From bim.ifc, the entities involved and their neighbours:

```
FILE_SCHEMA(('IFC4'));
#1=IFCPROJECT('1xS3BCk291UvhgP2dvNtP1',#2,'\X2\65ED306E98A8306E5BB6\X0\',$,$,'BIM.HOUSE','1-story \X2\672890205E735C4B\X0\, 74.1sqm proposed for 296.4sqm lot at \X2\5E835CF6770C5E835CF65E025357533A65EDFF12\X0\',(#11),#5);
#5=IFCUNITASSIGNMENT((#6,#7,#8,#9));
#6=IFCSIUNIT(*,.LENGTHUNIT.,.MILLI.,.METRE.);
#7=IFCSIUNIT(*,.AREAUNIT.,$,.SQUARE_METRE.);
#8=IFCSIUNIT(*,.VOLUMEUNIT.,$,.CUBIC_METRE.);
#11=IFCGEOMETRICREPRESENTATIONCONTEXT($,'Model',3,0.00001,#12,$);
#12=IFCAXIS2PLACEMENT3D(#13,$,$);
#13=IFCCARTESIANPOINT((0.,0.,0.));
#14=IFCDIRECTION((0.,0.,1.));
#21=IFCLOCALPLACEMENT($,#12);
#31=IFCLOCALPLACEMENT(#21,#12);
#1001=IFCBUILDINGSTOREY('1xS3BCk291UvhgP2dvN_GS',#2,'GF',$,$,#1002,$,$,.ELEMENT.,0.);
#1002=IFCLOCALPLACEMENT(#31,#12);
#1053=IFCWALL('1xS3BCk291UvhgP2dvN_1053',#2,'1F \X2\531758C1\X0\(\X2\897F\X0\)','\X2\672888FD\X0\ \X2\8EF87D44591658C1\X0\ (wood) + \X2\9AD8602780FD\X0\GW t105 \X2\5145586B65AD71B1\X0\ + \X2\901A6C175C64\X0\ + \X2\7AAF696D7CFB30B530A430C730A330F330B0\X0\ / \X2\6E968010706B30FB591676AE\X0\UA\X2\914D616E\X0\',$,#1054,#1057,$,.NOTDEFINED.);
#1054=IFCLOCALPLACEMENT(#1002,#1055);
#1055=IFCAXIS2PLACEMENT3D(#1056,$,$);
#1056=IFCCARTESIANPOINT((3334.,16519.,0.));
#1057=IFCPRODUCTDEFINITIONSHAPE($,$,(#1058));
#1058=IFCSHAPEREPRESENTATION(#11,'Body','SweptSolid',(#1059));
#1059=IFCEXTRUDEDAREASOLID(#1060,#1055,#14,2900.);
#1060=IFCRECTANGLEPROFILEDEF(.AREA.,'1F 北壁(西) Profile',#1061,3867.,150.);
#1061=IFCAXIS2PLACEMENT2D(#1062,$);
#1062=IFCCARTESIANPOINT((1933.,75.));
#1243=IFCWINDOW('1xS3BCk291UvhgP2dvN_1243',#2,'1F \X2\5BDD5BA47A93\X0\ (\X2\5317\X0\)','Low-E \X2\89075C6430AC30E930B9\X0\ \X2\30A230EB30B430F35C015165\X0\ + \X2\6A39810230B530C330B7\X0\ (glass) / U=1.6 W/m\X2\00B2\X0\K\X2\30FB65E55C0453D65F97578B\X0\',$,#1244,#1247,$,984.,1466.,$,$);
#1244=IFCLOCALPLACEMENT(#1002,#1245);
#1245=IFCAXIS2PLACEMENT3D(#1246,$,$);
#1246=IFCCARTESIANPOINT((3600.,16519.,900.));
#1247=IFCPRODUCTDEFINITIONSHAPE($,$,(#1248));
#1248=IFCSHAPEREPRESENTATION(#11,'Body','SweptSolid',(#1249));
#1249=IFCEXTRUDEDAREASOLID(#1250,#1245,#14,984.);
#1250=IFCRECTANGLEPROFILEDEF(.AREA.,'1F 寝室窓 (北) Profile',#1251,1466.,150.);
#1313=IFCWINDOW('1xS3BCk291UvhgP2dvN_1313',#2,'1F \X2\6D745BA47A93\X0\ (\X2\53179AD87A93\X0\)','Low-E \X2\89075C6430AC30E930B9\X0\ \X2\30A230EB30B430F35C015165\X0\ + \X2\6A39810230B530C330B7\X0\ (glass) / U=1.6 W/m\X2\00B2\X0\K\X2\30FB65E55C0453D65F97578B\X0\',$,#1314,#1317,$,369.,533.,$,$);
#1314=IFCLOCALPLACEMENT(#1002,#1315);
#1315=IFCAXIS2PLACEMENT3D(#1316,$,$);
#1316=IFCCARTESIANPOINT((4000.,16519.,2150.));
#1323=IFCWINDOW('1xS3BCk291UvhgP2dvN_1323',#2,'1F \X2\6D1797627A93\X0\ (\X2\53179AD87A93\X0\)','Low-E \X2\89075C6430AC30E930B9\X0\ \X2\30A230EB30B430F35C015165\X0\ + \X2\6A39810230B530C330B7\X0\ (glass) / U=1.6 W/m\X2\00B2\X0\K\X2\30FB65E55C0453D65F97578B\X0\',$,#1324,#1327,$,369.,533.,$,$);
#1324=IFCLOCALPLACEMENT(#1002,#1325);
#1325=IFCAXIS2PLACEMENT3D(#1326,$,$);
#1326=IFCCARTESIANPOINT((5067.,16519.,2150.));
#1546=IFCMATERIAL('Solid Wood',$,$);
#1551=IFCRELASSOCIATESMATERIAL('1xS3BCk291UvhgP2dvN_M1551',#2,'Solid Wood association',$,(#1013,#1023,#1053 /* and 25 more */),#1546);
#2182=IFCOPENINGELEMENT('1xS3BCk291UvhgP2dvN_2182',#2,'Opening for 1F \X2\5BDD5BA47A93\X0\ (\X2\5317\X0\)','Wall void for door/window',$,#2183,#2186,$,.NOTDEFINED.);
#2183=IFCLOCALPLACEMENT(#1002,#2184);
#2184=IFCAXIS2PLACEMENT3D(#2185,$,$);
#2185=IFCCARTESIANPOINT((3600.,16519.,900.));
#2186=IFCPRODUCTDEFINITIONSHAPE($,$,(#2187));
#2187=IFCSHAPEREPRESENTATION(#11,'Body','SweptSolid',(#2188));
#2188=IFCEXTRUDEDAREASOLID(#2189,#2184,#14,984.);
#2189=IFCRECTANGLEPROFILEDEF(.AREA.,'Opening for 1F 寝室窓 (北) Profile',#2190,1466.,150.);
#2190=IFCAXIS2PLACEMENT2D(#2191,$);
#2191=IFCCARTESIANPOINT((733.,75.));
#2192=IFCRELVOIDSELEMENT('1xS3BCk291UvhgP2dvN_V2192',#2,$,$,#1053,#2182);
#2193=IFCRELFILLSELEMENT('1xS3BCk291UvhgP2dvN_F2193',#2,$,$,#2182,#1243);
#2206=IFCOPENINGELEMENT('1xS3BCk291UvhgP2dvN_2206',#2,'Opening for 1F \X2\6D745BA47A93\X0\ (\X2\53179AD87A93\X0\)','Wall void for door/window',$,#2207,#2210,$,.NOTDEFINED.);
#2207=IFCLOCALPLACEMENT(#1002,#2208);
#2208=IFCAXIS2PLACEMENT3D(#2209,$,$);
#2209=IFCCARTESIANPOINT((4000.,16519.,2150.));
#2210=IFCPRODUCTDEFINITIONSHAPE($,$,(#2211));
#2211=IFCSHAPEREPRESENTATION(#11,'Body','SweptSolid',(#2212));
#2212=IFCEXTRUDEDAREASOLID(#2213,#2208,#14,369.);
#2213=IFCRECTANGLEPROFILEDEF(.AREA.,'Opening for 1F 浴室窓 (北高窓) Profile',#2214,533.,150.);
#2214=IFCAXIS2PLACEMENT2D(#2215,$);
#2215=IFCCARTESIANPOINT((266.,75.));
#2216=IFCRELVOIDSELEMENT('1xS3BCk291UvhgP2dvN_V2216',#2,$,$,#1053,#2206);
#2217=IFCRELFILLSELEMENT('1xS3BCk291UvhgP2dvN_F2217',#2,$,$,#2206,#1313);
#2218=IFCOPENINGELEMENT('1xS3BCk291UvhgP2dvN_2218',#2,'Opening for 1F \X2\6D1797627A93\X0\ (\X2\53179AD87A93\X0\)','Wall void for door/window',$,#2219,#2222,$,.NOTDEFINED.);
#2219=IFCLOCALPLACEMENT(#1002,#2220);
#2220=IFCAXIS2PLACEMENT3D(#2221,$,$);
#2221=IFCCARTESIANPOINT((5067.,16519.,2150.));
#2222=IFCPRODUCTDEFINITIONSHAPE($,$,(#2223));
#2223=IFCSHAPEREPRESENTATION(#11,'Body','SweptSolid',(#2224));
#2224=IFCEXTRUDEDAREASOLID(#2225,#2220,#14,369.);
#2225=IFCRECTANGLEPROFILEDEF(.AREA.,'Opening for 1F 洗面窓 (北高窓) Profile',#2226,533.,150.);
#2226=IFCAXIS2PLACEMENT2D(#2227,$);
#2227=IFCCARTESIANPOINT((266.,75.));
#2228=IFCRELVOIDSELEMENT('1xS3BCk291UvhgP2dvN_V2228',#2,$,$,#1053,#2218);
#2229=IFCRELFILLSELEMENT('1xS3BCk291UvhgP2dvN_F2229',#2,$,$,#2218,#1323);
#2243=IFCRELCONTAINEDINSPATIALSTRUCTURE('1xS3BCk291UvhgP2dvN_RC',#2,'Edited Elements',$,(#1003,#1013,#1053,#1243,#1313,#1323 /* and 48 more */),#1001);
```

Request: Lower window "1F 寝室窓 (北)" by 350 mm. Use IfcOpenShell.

```python
import numpy as np
import ifcopenshell
import ifcopenshell.api.geometry
import ifcopenshell.util.placement
import ifcopenshell.util.unit

model = ifcopenshell.open("bim.ifc")
unit_scale = ifcopenshell.util.unit.calculate_unit_scale(model)

window = model.by_guid("1xS3BCk291UvhgP2dvN_1243")
opening = window.FillsVoids[0].RelatingOpeningElement
dz = -0.35 / unit_scale

shift = np.array([0.0, 0.0, dz])
# The window is not placed relative to its opening, so move both.
for product in (opening, window):
    matrix = ifcopenshell.util.placement.get_local_placement(product.ObjectPlacement)
    matrix[:3, 3] += shift
    ifcopenshell.api.geometry.edit_object_placement(model, product=product, matrix=matrix, is_si=False)

print(f"moved by {dz * unit_scale:+.3f} m")

model.write("bim-out.ifc")
```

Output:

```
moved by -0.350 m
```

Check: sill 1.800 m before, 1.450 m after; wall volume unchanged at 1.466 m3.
